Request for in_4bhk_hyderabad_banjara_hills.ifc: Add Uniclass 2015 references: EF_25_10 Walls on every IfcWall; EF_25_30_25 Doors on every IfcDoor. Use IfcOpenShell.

First a look at what the model holds.

```python
import ifcopenshell

model = ifcopenshell.open("in_4bhk_hyderabad_banjara_hills.ifc")
print(model.schema)
print("classifications:", [c.Name for c in model.by_type("IfcClassification")])
for ifc_class in ("IfcDoor", "IfcRoof", "IfcStair", "IfcWall", "IfcWindow"):
    print(ifc_class, len(model.by_type(ifc_class)))
```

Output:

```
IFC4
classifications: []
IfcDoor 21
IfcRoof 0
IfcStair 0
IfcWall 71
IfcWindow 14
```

```python
import ifcopenshell
import ifcopenshell.api.classification

model = ifcopenshell.open("in_4bhk_hyderabad_banjara_hills.ifc")

system = ifcopenshell.api.classification.add_classification(model, classification="Uniclass 2015")

codes = {
    "IfcWall": ("EF_25_10", "Walls"),
    "IfcDoor": ("EF_25_30_25", "Doors"),
}
for ifc_class, (code, name) in codes.items():
    products = model.by_type(ifc_class)
    ifcopenshell.api.classification.add_reference(
        model, products=products, classification=system, identification=code, name=name
    )
    print(code, len(products))

model.write("in_4bhk_hyderabad_banjara_hills_v2.ifc")
```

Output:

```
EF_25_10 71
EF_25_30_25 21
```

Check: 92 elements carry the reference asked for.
